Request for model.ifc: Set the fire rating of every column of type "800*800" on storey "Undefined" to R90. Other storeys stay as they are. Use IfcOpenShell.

First a look at what the model holds.

```python
import ifcopenshell
import ifcopenshell.util.element

model = ifcopenshell.open("model.ifc")
print(model.schema)
storey = next(s for s in model.by_type("IfcBuildingStorey") if s.Name == "Undefined")
columns = [e for e in ifcopenshell.util.element.get_decomposition(storey) if e.is_a("IfcColumn")]
seen = {}
for e in columns:
    element_type = ifcopenshell.util.element.get_type(e)
    key = (element_type.Name if element_type != e and element_type else None, ifcopenshell.util.element.get_pset(e, "Pset_ColumnCommon", "FireRating"))
    seen[key] = seen.get(key, 0) + 1
for (name, value), count in sorted(seen.items(), key=str):
    print(count, "x", name, "|", value)
```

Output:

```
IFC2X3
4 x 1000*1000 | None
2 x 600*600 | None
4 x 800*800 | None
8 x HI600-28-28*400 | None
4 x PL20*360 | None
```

```python
import ifcopenshell
import ifcopenshell.api.pset
import ifcopenshell.util.element

model = ifcopenshell.open("model.ifc")

storey = next(s for s in model.by_type("IfcBuildingStorey") if s.Name == "Undefined")
columns = [e for e in ifcopenshell.util.element.get_decomposition(storey) if e.is_a("IfcColumn")]

count = 0
for e in columns:
    element_type = ifcopenshell.util.element.get_type(e)
    if element_type in (None, e) or element_type.Name != "800*800":
        continue
    found = ifcopenshell.util.element.get_pset(e, "Pset_ColumnCommon", should_inherit=False)
    if found:
        pset = model.by_id(found["id"])
        if len(ifcopenshell.util.element.get_elements_by_pset(pset)) > 1:
            pset = ifcopenshell.api.pset.unshare_pset(model, products=[e], pset=pset)[0]
    else:
        pset = ifcopenshell.api.pset.add_pset(model, product=e, name="Pset_ColumnCommon")
    ifcopenshell.api.pset.edit_pset(model, pset=pset, properties={"FireRating": "R90"})
    count += 1

print(count, "columns updated")

model.write("model_v2.ifc")
```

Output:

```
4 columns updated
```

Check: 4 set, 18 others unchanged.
